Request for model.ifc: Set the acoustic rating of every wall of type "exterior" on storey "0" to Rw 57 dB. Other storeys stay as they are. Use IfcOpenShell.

First a look at what the model holds.

```python
import ifcopenshell
import ifcopenshell.util.element

model = ifcopenshell.open("model.ifc")
print(model.schema)
storey = next(s for s in model.by_type("IfcBuildingStorey") if s.Name == "0")
walls = [e for e in ifcopenshell.util.element.get_decomposition(storey) if e.is_a("IfcWall")]
seen = {}
for e in walls:
    element_type = ifcopenshell.util.element.get_type(e)
    key = (element_type.Name if element_type != e and element_type else None, ifcopenshell.util.element.get_pset(e, "Pset_WallCommon", "AcousticRating"))
    seen[key] = seen.get(key, 0) + 1
for (name, value), count in sorted(seen.items(), key=str):
    print(count, "x", name, "|", value)
```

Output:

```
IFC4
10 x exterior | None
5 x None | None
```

```python
import ifcopenshell
import ifcopenshell.api.pset
import ifcopenshell.util.element

model = ifcopenshell.open("model.ifc")

storey = next(s for s in model.by_type("IfcBuildingStorey") if s.Name == "0")
walls = [e for e in ifcopenshell.util.element.get_decomposition(storey) if e.is_a("IfcWall")]

count = 0
for e in walls:
    element_type = ifcopenshell.util.element.get_type(e)
    if element_type in (None, e) or element_type.Name != "exterior":
        continue
    # add_pset returns the element's existing set when there is one.
    pset = ifcopenshell.api.pset.add_pset(model, product=e, name="Pset_WallCommon")
    ifcopenshell.api.pset.edit_pset(model, pset=pset, properties={"AcousticRating": "Rw 57 dB"})
    count += 1

print(count, "walls updated")

model.write("model-out.ifc")
```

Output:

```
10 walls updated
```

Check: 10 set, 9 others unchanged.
